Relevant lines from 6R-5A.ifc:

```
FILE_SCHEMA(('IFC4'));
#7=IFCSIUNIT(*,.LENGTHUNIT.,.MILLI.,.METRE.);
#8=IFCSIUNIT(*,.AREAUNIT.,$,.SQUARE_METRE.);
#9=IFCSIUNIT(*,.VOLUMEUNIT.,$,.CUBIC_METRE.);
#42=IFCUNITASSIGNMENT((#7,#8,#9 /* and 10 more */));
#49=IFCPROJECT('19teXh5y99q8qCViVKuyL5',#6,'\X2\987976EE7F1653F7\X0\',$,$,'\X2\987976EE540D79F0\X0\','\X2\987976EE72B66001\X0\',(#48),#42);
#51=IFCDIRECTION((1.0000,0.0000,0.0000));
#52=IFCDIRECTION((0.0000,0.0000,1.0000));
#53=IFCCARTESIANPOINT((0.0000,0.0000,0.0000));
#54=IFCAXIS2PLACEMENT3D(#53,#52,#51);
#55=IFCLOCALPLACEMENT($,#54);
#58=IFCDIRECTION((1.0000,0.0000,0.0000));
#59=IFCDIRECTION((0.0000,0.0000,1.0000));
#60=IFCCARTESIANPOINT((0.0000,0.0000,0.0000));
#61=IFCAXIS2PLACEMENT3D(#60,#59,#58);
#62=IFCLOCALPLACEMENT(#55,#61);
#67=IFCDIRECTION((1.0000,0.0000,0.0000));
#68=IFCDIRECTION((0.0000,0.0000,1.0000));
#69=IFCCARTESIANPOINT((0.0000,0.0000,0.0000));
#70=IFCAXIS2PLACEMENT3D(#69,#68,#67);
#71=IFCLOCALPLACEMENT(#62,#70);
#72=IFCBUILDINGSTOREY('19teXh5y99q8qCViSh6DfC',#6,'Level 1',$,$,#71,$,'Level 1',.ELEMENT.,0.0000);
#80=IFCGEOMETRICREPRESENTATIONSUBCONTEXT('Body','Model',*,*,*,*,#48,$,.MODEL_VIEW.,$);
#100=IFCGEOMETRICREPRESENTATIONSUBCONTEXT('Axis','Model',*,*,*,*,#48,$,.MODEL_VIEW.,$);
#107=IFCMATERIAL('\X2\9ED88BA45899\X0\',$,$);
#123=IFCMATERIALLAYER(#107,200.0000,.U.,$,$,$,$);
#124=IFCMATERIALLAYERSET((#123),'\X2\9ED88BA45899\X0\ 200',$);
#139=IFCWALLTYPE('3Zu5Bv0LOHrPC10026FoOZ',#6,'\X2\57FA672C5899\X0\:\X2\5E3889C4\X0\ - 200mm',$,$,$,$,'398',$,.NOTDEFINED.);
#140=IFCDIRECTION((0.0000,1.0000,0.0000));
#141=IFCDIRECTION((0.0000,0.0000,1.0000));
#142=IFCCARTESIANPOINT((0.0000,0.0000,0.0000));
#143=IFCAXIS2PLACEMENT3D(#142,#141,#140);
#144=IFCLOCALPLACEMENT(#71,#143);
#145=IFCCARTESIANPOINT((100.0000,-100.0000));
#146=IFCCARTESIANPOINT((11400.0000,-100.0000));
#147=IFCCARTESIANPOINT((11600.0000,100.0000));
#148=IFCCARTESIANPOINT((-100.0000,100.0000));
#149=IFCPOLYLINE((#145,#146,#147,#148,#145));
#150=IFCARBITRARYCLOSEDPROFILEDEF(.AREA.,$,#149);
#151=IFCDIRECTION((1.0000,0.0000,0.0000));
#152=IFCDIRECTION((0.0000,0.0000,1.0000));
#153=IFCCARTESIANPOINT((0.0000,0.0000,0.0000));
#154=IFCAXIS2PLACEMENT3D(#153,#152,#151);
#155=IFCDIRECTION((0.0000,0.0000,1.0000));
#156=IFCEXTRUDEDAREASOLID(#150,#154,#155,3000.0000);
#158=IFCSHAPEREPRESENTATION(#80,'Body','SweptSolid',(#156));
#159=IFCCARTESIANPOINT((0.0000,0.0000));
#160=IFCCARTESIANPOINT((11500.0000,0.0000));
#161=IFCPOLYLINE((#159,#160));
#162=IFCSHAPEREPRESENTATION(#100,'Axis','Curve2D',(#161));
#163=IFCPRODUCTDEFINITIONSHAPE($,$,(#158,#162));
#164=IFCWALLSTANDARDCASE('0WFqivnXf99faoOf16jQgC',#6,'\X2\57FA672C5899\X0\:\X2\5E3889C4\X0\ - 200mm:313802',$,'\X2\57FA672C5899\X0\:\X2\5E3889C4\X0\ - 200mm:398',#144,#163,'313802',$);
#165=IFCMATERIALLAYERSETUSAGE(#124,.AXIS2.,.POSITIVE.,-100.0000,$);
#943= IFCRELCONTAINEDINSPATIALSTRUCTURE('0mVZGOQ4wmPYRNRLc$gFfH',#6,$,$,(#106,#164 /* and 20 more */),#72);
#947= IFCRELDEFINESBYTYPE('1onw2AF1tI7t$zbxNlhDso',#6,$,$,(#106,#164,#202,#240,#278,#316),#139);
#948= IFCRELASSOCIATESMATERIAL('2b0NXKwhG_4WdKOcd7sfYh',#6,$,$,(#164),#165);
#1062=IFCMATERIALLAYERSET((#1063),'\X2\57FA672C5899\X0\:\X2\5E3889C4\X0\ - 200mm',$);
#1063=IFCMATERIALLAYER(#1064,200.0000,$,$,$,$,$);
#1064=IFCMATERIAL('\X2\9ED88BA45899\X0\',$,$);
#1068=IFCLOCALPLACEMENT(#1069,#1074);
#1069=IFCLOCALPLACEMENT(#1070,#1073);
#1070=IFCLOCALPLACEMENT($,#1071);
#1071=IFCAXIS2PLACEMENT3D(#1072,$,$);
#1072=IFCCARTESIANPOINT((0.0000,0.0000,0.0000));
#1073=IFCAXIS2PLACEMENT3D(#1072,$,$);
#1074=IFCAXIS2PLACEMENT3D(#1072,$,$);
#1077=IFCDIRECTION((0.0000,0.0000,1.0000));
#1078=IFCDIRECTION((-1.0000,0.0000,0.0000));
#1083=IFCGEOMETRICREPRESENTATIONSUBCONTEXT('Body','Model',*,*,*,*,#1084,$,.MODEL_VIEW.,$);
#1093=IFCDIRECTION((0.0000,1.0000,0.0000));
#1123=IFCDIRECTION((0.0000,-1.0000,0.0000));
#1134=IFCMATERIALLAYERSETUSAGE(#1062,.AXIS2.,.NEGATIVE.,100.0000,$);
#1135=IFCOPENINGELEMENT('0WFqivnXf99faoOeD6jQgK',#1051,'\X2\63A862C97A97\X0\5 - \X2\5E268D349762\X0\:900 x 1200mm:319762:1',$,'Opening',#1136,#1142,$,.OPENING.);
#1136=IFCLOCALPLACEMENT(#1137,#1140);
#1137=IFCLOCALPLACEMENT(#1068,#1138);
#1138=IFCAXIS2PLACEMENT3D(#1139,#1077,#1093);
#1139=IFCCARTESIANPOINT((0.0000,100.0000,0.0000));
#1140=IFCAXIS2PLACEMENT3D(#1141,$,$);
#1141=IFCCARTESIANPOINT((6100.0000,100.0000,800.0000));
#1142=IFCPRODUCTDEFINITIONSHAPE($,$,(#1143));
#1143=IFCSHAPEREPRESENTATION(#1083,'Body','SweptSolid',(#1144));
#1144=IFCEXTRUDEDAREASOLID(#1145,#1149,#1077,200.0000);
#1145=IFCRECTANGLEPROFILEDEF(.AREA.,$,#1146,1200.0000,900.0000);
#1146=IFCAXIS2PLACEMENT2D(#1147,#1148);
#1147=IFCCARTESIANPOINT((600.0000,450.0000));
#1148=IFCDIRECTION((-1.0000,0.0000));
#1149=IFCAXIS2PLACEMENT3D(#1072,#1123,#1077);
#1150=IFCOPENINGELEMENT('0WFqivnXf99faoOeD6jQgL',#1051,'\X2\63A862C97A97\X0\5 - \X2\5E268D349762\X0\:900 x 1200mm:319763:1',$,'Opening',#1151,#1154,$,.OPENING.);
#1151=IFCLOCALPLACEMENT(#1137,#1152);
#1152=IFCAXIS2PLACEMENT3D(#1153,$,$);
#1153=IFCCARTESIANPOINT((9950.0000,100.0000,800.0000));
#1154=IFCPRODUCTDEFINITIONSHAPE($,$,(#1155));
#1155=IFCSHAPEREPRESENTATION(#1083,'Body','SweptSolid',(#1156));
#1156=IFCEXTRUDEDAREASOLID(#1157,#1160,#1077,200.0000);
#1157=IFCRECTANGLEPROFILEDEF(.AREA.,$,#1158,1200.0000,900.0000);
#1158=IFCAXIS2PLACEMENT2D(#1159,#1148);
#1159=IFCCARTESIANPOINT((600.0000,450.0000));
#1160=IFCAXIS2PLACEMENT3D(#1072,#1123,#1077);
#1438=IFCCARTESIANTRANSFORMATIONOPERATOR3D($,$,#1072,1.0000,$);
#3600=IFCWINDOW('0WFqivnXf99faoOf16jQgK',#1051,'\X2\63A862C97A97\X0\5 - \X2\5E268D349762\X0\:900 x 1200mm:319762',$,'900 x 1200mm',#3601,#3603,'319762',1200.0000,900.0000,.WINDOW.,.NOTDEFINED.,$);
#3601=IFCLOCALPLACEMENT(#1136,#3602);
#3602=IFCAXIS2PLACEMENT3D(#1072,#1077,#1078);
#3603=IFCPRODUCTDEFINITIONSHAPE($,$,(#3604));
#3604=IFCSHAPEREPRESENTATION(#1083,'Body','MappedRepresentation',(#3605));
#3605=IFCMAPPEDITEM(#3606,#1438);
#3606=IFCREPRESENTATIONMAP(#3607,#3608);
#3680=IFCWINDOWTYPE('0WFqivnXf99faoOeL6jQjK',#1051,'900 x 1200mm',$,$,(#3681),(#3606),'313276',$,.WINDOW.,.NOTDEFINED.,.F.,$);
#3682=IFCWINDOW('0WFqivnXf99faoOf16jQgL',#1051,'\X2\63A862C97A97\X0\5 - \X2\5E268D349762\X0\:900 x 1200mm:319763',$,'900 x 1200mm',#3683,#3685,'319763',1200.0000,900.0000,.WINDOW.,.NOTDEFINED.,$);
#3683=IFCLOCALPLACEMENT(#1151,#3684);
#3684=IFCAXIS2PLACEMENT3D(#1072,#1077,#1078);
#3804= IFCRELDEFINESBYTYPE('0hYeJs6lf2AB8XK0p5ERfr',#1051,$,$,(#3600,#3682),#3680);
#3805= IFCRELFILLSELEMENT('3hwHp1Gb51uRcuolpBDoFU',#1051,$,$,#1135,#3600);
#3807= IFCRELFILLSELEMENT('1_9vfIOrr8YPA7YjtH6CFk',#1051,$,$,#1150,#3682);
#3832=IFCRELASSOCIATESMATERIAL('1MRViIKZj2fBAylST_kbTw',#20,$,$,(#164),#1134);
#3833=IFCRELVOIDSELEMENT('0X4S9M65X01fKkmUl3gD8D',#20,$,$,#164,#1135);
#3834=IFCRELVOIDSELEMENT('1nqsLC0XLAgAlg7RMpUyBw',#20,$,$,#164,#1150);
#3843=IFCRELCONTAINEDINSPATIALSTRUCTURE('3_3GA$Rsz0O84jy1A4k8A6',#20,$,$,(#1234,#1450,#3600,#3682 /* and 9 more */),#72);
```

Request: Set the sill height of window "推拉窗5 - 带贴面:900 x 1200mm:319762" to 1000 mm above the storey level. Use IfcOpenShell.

```python
import numpy as np
import ifcopenshell
import ifcopenshell.api.geometry
import ifcopenshell.geom
import ifcopenshell.util.element
import ifcopenshell.util.placement
import ifcopenshell.util.shape
import ifcopenshell.util.unit

model = ifcopenshell.open("6R-5A.ifc")
unit_scale = ifcopenshell.util.unit.calculate_unit_scale(model)

window = model.by_guid("0WFqivnXf99faoOf16jQgK")
opening = window.FillsVoids[0].RelatingOpeningElement
storey = ifcopenshell.util.element.get_container(window, ifc_class="IfcBuildingStorey")
level = ifcopenshell.util.placement.get_local_placement(storey.ObjectPlacement)[2, 3]

# The opening's origin need not be at the sill, so measure its lowest point.
shape = ifcopenshell.geom.create_shape(ifcopenshell.geom.settings(), opening)
bottom = ifcopenshell.util.shape.get_shape_bottom_elevation(shape, shape.geometry) / unit_scale
dz = level + 1 / unit_scale - bottom

shift = np.array([0.0, 0.0, dz])
# The window is placed relative to its opening, so it follows when the opening moves.
matrix = ifcopenshell.util.placement.get_local_placement(opening.ObjectPlacement)
matrix[:3, 3] += shift
ifcopenshell.api.geometry.edit_object_placement(
    model, product=opening, matrix=matrix, is_si=False, should_transform_children=True
)

print(f"moved by {dz * unit_scale:+.3f} m")

model.write("6R-5A-out.ifc")
```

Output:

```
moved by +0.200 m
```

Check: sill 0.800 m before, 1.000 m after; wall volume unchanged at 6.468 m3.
